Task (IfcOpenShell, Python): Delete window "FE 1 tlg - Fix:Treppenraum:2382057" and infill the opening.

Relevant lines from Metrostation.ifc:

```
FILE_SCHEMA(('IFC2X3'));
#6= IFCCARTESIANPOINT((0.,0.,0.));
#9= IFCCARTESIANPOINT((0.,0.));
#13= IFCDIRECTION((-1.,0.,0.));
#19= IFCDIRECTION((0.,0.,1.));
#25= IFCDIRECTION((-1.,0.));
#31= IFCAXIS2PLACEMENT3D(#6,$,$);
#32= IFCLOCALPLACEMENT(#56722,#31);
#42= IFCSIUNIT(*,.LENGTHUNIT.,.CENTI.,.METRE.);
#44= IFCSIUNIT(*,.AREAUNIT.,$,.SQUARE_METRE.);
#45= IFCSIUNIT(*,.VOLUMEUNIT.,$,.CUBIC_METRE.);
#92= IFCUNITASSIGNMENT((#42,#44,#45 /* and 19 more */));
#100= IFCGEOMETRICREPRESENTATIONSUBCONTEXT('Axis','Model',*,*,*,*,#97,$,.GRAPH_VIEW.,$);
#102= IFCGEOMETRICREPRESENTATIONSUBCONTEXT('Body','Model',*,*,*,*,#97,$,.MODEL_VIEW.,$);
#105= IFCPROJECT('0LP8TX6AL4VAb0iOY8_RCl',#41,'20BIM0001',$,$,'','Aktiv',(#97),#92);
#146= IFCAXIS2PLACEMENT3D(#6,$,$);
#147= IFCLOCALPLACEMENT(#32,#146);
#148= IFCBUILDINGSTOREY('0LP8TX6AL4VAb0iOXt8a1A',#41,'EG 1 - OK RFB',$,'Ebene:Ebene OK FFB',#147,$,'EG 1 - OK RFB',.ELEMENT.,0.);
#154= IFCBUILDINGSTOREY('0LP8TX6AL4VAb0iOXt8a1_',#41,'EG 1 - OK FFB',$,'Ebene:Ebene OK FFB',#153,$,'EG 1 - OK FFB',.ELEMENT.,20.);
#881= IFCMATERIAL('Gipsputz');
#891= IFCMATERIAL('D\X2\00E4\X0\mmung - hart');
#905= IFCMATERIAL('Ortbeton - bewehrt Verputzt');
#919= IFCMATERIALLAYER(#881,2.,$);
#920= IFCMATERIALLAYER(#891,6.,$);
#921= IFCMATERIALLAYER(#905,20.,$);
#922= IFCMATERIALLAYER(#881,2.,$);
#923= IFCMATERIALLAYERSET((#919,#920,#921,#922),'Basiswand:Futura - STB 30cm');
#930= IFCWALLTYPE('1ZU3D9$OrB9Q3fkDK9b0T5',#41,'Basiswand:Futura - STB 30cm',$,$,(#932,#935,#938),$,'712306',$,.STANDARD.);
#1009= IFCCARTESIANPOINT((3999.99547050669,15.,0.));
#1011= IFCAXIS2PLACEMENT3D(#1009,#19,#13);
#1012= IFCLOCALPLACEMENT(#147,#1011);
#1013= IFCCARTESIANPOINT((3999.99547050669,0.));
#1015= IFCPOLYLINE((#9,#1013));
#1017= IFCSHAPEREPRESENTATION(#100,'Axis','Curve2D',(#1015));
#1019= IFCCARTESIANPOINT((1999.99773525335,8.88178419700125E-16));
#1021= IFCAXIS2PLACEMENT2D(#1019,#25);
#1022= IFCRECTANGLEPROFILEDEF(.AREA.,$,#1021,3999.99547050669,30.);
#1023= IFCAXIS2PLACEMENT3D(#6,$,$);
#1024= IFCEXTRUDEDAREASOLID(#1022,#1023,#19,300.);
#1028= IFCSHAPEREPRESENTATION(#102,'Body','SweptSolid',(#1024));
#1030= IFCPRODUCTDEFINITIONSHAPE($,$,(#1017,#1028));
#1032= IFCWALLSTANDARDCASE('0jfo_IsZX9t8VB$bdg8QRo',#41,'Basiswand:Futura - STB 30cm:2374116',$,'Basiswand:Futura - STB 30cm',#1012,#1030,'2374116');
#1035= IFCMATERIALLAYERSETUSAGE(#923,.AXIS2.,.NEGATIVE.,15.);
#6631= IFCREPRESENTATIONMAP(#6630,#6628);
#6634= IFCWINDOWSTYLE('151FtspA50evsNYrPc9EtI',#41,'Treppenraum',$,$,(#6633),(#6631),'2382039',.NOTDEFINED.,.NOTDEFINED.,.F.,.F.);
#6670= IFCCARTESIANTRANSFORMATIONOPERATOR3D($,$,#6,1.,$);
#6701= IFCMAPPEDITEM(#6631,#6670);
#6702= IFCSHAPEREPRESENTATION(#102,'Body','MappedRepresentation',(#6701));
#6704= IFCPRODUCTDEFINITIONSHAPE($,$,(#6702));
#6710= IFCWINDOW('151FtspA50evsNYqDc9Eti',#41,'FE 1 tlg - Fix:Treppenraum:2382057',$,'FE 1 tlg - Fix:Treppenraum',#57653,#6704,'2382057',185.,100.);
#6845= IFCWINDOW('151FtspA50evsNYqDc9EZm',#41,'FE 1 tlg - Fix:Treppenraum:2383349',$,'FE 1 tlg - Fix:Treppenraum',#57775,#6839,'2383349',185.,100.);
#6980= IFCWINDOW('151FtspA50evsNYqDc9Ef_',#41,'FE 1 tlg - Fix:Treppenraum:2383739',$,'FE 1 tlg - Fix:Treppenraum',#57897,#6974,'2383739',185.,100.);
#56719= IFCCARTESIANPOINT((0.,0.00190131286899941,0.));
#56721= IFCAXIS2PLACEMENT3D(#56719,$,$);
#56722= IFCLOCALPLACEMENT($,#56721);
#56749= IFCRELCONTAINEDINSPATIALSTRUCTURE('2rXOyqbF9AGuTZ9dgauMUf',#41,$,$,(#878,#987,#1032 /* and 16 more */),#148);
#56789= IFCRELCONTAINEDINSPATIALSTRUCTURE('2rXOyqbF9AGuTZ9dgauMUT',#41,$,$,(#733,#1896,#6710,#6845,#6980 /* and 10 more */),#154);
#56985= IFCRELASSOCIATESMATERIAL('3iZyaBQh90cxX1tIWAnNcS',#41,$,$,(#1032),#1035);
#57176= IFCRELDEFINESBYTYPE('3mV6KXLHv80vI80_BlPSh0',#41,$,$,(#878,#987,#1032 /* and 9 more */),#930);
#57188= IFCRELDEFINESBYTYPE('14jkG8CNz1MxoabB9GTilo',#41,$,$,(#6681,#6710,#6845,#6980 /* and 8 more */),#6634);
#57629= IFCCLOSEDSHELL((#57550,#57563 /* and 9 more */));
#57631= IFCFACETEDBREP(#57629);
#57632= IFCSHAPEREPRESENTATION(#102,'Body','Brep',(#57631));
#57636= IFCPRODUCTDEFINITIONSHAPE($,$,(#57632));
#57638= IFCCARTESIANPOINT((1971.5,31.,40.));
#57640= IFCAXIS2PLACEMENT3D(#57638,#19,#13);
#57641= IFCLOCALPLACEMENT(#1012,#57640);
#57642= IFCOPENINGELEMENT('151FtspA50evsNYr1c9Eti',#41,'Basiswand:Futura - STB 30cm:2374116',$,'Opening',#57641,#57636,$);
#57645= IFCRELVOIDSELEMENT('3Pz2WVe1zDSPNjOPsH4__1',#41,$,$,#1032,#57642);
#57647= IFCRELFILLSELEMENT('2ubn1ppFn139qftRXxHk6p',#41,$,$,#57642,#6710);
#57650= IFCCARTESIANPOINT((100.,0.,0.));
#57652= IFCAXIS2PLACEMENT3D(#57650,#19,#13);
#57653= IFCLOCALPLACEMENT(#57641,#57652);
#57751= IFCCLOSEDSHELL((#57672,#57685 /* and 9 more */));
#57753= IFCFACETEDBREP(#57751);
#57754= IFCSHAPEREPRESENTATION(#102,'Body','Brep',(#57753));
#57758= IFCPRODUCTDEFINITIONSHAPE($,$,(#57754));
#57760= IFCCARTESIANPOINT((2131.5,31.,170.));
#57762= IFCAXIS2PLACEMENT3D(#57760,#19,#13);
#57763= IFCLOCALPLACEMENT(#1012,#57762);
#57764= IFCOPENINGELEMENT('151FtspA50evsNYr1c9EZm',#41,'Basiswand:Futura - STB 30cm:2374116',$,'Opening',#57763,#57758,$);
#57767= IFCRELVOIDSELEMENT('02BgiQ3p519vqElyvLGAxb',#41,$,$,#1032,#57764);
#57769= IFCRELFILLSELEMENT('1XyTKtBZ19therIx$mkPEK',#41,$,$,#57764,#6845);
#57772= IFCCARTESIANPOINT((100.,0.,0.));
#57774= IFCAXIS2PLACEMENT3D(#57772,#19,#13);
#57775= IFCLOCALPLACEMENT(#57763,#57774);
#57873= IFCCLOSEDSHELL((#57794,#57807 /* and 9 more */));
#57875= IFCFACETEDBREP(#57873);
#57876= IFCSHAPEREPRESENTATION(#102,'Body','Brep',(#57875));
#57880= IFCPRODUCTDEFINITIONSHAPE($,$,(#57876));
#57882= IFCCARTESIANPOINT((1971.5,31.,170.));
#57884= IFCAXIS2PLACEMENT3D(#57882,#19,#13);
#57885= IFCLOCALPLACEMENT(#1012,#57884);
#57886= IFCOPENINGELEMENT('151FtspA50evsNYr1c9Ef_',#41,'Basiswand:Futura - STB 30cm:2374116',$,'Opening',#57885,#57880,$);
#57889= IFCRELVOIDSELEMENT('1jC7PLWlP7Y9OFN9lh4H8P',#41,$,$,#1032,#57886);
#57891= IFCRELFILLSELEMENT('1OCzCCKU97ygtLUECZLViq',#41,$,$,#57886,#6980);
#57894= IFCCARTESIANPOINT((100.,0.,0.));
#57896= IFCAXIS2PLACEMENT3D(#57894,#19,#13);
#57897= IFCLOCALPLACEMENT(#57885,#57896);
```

```python
import ifcopenshell
import ifcopenshell.api.feature
import ifcopenshell.api.root
import ifcopenshell.geom
import ifcopenshell.util.shape

model = ifcopenshell.open("Metrostation.ifc")
settings = ifcopenshell.geom.settings()


def volume(element):
    """Net volume in cubic metres, openings subtracted."""
    shape = ifcopenshell.geom.create_shape(settings, element)
    return ifcopenshell.util.shape.get_volume(shape.geometry)


window = model.by_guid("151FtspA50evsNYqDc9Eti")
opening = window.FillsVoids[0].RelatingOpeningElement
wall = opening.VoidsElements[0].RelatingBuildingElement
before = volume(wall)

ifcopenshell.api.root.remove_product(model, product=window)
ifcopenshell.api.feature.remove_feature(model, feature=opening)

after = volume(wall)

print(f"wall volume {before:.3f} -> {after:.3f} m3")

model.write("Metrostation_rev.ifc")
```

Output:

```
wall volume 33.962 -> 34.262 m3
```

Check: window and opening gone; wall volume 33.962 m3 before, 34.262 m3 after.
